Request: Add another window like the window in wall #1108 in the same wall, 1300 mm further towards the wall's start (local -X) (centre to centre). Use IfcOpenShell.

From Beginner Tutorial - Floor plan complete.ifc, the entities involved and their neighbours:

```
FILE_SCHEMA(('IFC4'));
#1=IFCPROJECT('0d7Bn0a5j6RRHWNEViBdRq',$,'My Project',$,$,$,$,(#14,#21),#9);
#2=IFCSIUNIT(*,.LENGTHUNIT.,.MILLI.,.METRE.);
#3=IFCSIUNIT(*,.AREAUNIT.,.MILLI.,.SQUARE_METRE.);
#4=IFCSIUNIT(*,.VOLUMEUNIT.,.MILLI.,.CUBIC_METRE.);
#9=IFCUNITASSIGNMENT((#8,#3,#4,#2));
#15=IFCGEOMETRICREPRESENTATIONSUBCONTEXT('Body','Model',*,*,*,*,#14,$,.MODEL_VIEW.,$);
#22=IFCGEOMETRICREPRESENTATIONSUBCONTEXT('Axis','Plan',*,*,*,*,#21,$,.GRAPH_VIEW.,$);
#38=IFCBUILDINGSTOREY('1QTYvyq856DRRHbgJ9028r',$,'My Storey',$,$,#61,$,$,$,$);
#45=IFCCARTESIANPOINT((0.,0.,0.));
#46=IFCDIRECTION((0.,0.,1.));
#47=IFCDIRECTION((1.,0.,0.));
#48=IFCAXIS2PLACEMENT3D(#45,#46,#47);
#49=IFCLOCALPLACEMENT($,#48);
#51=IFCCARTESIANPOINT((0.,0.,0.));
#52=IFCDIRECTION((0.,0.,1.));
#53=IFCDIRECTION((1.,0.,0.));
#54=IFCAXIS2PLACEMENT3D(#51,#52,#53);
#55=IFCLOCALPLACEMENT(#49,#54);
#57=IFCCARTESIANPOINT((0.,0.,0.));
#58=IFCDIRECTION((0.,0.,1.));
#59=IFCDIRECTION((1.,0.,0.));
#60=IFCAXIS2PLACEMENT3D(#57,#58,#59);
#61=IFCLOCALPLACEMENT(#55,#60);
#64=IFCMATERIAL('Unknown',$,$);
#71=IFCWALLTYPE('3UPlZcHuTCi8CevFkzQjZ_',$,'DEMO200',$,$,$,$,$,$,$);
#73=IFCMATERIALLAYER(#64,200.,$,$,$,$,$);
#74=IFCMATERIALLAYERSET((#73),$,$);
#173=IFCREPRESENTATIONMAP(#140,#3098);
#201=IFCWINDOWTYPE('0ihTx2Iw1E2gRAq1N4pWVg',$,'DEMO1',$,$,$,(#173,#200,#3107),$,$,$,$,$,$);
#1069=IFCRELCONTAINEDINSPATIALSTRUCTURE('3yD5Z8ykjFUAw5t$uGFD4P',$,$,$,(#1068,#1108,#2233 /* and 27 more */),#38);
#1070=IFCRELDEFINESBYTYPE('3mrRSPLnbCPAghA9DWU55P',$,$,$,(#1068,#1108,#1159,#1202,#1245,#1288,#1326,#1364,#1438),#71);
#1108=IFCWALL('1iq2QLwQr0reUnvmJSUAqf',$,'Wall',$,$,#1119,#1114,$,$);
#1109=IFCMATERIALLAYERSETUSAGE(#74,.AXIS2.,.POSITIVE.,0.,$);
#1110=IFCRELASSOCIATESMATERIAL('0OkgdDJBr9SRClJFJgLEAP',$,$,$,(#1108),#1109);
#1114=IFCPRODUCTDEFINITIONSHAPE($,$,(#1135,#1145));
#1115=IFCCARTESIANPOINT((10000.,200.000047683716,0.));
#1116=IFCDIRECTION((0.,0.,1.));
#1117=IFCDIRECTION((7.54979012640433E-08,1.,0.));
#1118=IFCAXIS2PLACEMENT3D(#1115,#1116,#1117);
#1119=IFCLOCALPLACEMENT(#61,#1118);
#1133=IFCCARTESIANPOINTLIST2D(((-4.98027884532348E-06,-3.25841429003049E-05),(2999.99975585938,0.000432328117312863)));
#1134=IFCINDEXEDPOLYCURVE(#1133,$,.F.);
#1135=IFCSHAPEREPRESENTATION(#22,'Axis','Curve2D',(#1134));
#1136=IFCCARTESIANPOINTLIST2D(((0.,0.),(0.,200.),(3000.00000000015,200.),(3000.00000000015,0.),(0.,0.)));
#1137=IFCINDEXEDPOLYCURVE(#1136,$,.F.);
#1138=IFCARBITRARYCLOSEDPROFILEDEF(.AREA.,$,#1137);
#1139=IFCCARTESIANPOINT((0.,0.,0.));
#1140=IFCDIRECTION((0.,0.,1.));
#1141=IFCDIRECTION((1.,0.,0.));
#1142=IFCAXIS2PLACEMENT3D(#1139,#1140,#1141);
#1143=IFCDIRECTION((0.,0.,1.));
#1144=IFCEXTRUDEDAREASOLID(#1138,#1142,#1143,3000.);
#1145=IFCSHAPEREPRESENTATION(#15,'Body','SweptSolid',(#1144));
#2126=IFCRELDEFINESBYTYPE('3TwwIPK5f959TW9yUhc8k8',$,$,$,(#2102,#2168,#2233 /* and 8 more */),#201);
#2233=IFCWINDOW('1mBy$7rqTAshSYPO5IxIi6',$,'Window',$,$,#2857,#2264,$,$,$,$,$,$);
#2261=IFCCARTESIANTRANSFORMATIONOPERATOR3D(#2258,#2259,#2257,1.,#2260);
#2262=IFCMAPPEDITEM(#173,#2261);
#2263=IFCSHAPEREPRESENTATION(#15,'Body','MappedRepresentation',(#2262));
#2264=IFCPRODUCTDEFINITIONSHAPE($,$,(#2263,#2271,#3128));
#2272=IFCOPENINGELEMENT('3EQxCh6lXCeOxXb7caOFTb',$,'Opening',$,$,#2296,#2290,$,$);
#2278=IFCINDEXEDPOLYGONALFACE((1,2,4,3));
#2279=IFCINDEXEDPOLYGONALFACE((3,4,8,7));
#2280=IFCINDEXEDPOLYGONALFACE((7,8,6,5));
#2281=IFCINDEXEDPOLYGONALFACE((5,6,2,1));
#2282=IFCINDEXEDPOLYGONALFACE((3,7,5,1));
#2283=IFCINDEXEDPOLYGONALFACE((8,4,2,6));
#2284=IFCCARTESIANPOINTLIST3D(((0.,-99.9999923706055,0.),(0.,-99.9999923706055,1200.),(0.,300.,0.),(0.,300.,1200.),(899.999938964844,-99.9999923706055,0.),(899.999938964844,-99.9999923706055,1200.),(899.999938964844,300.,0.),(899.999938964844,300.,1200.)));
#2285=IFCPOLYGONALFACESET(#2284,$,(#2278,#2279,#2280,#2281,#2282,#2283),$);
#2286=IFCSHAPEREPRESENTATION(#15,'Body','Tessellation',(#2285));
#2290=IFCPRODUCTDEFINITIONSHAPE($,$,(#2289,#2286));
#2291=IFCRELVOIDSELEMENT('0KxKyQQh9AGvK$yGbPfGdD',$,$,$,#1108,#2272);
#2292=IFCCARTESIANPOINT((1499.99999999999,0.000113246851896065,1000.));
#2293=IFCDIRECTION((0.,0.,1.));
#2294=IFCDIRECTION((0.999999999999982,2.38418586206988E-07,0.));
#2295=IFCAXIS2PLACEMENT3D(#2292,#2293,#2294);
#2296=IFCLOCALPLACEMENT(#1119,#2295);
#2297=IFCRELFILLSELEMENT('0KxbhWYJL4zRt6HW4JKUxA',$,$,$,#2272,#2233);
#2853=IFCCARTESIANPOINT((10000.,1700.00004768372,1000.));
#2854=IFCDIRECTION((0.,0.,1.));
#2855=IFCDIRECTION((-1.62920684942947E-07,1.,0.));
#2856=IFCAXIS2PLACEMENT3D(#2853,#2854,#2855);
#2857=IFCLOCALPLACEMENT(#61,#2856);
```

```python
import ifcopenshell
import ifcopenshell.api.feature
import ifcopenshell.api.geometry
import ifcopenshell.api.root
import ifcopenshell.geom
import ifcopenshell.util.element
import ifcopenshell.util.placement
import ifcopenshell.util.shape
import ifcopenshell.util.unit

model = ifcopenshell.open("Beginner Tutorial - Floor plan complete.ifc")
unit_scale = ifcopenshell.util.unit.calculate_unit_scale(model)
settings = ifcopenshell.geom.settings()


def volume(element):
    """Net volume in cubic metres, openings subtracted."""
    shape = ifcopenshell.geom.create_shape(settings, element)
    return ifcopenshell.util.shape.get_volume(shape.geometry)


window = model.by_id(2233)
opening = window.FillsVoids[0].RelatingOpeningElement
wall = opening.VoidsElements[0].RelatingBuildingElement
before = volume(wall)
shift = ifcopenshell.util.placement.get_local_placement(wall.ObjectPlacement)[:3, 0] * -1.3 / unit_scale

# copy_class copies the void relationship, type, container and properties, but no geometry.
new_opening = ifcopenshell.api.root.copy_class(model, product=opening)
new_opening.Representation = ifcopenshell.util.element.copy_deep(
    model, opening.Representation, exclude=["IfcGeometricRepresentationContext", "IfcRepresentationMap"]
)
new_window = ifcopenshell.api.root.copy_class(model, product=window)
new_window.Representation = ifcopenshell.util.element.copy_deep(
    model, window.Representation, exclude=["IfcGeometricRepresentationContext", "IfcRepresentationMap"]
)
ifcopenshell.api.feature.add_filling(model, opening=new_opening, element=new_window)

for old, new in ((opening, new_opening), (window, new_window)):
    matrix = ifcopenshell.util.placement.get_local_placement(old.ObjectPlacement)
    matrix[:3, 3] += shift
    ifcopenshell.api.geometry.edit_object_placement(model, product=new, matrix=matrix, is_si=False)

after = volume(wall)

print(f"wall volume {before:.3f} -> {after:.3f} m3")

model.write("Beginner Tutorial - Floor plan complete_updated.ifc")
```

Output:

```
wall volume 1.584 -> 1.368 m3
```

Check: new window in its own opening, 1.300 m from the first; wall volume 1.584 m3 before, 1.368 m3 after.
